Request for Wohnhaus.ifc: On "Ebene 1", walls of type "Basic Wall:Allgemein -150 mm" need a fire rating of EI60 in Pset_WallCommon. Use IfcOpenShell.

First a look at what the model holds.

```python
import ifcopenshell
import ifcopenshell.util.element

model = ifcopenshell.open("Wohnhaus.ifc")
print(model.schema)
storey = next(s for s in model.by_type("IfcBuildingStorey") if s.Name == "Ebene 1")
walls = [e for e in ifcopenshell.util.element.get_decomposition(storey) if e.is_a("IfcWall")]
seen = {}
for e in walls:
    element_type = ifcopenshell.util.element.get_type(e)
    key = (element_type.Name if element_type != e and element_type else None, ifcopenshell.util.element.get_pset(e, "Pset_WallCommon", "FireRating"))
    seen[key] = seen.get(key, 0) + 1
for (name, value), count in sorted(seen.items(), key=str):
    print(count, "x", name, "|", value)
```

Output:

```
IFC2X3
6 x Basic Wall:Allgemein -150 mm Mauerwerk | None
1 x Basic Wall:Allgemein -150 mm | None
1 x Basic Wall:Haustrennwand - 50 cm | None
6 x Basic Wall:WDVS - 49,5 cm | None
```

```python
import ifcopenshell
import ifcopenshell.api.pset
import ifcopenshell.util.element

model = ifcopenshell.open("Wohnhaus.ifc")

storey = next(s for s in model.by_type("IfcBuildingStorey") if s.Name == "Ebene 1")
walls = [e for e in ifcopenshell.util.element.get_decomposition(storey) if e.is_a("IfcWall")]

count = 0
for e in walls:
    element_type = ifcopenshell.util.element.get_type(e)
    if element_type in (None, e) or element_type.Name != "Basic Wall:Allgemein -150 mm":
        continue
    # add_pset returns the element's existing set when there is one.
    pset = ifcopenshell.api.pset.add_pset(model, product=e, name="Pset_WallCommon")
    ifcopenshell.api.pset.edit_pset(model, pset=pset, properties={"FireRating": "EI60"})
    count += 1

print(count, "walls updated")

model.write("Wohnhaus_rev.ifc")
```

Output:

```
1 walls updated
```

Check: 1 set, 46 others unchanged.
